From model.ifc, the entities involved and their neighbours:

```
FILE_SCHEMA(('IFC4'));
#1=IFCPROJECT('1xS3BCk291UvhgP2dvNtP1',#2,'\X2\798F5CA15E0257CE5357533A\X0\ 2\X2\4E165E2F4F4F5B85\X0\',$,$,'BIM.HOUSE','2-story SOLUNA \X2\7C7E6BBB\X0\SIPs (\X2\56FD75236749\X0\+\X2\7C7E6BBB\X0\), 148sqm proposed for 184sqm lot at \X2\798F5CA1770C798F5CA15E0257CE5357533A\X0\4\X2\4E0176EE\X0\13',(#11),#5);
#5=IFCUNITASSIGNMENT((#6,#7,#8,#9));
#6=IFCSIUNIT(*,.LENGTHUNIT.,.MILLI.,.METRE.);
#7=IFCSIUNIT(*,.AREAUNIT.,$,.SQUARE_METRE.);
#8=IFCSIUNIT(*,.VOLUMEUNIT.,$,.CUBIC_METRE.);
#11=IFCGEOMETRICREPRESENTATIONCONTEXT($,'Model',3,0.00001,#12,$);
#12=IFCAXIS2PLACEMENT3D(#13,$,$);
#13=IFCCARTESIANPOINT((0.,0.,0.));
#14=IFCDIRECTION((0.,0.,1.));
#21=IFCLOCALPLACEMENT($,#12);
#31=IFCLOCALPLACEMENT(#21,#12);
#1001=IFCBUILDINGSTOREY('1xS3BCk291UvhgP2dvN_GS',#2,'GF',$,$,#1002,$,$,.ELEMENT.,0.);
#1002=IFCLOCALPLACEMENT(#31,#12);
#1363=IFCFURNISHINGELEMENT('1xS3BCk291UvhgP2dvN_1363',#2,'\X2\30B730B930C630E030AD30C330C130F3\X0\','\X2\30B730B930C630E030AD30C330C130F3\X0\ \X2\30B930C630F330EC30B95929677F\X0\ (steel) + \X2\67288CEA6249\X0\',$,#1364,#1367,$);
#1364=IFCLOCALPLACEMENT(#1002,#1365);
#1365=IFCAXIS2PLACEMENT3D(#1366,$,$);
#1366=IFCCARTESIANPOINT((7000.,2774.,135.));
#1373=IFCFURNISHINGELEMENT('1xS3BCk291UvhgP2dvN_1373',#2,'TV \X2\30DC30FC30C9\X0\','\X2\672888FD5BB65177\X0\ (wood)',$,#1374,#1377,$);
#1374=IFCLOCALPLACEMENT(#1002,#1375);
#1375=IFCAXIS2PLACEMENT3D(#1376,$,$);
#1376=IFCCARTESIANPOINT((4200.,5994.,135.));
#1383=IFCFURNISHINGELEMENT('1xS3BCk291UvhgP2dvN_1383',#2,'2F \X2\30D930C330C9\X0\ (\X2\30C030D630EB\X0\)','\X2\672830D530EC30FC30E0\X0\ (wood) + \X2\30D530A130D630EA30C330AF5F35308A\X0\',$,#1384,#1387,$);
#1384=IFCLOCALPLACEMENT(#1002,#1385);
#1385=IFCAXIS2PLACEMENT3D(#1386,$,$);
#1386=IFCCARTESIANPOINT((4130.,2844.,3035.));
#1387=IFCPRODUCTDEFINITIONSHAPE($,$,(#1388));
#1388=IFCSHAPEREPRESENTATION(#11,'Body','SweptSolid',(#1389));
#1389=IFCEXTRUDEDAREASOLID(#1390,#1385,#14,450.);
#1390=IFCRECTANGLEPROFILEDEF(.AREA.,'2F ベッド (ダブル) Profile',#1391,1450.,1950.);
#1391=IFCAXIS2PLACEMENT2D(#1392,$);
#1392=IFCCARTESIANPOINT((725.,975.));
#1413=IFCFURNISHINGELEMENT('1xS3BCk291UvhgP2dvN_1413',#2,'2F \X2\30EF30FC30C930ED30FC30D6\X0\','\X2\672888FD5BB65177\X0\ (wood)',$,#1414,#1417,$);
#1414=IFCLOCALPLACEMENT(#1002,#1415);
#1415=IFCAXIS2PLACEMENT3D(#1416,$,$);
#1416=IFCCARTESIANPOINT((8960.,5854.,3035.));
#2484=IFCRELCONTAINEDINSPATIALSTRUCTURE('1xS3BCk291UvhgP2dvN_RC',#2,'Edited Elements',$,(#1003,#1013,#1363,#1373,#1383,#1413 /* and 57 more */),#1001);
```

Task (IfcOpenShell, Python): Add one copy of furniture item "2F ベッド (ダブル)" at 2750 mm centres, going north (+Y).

```python
import numpy as np
import ifcopenshell
import ifcopenshell.api.geometry
import ifcopenshell.api.root
import ifcopenshell.util.element
import ifcopenshell.util.placement
import ifcopenshell.util.unit

model = ifcopenshell.open("model.ifc")
unit_scale = ifcopenshell.util.unit.calculate_unit_scale(model)


def reuse_history(source, copy):
    """copy_class also copies each property set's owner history, people and application; keep the originals."""
    for rel in copy.IsDefinedBy:
        if rel.is_a("IfcRelDefinesByProperties") and (history := rel.RelatingPropertyDefinition.OwnerHistory):
            rel.RelatingPropertyDefinition.OwnerHistory = source.OwnerHistory
            ifcopenshell.util.element.remove_deep2(model, history)


source = model.by_guid("1xS3BCk291UvhgP2dvN_1383")
base = ifcopenshell.util.placement.get_local_placement(source.ObjectPlacement)
step = np.array([0.0, 1.0, 0.0]) * 2.75 / unit_scale

for i in range(1, 2):
    copy = ifcopenshell.api.root.copy_class(model, product=source)
    copy.Representation = ifcopenshell.util.element.copy_deep(
        model, source.Representation, exclude=["IfcGeometricRepresentationContext", "IfcRepresentationMap"]
    )
    reuse_history(source, copy)
    matrix = base.copy()
    matrix[:3, 3] += i * step
    print("added at", matrix[:3, 3].round(3) + 0.0)
    ifcopenshell.api.geometry.edit_object_placement(model, product=copy, matrix=matrix, is_si=False)

model.write("model_updated.ifc")
```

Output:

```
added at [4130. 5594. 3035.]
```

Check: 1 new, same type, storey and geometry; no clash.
